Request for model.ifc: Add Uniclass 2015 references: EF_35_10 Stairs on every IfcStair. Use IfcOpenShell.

First a look at what the model holds.

```python
import ifcopenshell

model = ifcopenshell.open("model.ifc")
print(model.schema)
print("classifications:", [c.Name for c in model.by_type("IfcClassification")])
for ifc_class in ("IfcDoor", "IfcRoof", "IfcStair", "IfcWall", "IfcWindow"):
    print(ifc_class, len(model.by_type(ifc_class)))
```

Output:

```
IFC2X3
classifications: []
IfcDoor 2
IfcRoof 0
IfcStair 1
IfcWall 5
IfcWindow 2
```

```python
import ifcopenshell
import ifcopenshell.api.classification

model = ifcopenshell.open("model.ifc")

# IFC2X3 requires Source and Edition and has no link from the project to the system.
system = model.create_entity("IfcClassification", Source="NBS", Edition="2015", Name="Uniclass 2015")

codes = {
    "IfcStair": ("EF_35_10", "Stairs"),
}
for ifc_class, (code, name) in codes.items():
    products = model.by_type(ifc_class)
    ifcopenshell.api.classification.add_reference(
        model, products=products, classification=system, identification=code, name=name
    )
    print(code, len(products))

model.write("model_v2.ifc")
```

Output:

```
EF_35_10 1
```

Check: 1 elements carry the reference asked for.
